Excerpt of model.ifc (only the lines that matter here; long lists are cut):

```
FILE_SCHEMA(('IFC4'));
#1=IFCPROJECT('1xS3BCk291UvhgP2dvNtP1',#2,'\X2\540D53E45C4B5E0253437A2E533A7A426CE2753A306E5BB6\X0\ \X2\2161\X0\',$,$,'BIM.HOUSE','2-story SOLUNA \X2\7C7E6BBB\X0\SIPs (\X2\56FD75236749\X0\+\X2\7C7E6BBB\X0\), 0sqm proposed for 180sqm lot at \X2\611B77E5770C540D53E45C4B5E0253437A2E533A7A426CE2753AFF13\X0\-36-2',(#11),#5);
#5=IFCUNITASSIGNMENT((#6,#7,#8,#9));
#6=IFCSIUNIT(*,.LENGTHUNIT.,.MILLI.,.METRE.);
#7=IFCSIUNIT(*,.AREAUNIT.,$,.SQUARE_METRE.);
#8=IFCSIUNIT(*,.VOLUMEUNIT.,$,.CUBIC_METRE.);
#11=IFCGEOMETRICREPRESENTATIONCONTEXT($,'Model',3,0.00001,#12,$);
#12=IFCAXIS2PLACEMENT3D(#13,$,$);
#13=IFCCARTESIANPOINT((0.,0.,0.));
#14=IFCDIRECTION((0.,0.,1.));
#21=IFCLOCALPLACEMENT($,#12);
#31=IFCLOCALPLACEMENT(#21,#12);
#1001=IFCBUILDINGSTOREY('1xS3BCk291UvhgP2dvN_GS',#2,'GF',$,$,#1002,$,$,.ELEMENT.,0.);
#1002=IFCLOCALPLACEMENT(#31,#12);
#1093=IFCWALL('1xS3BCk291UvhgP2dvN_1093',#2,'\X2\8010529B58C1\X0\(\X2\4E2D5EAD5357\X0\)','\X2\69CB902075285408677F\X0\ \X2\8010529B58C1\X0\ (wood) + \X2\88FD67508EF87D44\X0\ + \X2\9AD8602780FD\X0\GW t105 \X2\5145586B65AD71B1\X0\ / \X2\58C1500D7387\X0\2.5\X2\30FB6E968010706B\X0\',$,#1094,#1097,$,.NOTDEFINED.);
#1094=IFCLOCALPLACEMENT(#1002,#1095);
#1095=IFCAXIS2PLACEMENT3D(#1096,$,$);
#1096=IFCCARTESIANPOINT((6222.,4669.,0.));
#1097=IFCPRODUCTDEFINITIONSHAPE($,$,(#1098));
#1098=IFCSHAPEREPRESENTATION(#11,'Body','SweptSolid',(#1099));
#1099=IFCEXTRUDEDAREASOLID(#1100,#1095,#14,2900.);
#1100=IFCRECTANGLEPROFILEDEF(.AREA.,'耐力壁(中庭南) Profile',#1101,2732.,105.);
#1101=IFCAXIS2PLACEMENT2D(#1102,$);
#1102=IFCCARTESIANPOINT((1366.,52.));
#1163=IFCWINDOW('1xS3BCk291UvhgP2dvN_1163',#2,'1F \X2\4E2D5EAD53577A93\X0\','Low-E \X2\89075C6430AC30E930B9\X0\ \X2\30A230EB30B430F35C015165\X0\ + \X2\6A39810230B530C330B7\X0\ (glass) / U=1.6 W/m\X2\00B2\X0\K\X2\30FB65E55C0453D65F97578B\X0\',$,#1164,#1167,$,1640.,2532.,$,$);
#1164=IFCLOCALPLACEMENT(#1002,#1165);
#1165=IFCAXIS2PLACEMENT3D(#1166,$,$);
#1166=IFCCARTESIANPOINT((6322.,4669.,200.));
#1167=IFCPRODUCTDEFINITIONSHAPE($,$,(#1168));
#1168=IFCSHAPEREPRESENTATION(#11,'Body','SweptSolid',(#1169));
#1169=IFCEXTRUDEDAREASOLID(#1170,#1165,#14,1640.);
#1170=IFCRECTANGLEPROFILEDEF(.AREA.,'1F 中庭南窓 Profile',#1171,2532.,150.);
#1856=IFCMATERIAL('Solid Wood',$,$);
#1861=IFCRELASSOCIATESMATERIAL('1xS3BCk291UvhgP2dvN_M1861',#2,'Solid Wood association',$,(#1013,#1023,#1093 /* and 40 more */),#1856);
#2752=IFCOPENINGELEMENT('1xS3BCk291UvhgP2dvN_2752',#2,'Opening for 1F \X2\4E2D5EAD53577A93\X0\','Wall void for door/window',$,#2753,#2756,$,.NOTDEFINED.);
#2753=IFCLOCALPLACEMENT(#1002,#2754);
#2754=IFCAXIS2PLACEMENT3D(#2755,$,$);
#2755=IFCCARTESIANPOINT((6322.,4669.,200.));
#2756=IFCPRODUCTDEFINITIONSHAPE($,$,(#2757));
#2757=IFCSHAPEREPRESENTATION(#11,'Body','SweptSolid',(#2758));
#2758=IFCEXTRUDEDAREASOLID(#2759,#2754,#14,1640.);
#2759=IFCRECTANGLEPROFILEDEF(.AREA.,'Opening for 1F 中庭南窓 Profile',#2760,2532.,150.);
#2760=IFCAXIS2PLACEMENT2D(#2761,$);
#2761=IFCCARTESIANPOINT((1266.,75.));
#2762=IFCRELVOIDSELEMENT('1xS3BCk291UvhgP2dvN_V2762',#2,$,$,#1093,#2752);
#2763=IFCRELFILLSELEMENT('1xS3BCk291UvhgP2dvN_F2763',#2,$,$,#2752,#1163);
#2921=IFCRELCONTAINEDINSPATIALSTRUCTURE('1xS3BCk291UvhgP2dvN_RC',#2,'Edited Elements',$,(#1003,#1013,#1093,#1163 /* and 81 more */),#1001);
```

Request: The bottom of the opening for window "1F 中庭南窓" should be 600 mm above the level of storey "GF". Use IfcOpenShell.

```python
import numpy as np
import ifcopenshell
import ifcopenshell.api.geometry
import ifcopenshell.geom
import ifcopenshell.util.element
import ifcopenshell.util.placement
import ifcopenshell.util.shape
import ifcopenshell.util.unit

model = ifcopenshell.open("model.ifc")
unit_scale = ifcopenshell.util.unit.calculate_unit_scale(model)

window = model.by_id(1163)
opening = window.FillsVoids[0].RelatingOpeningElement
storey = ifcopenshell.util.element.get_container(window, ifc_class="IfcBuildingStorey")
level = ifcopenshell.util.placement.get_local_placement(storey.ObjectPlacement)[2, 3]

# The opening's origin need not be at the sill, so measure its lowest point.
shape = ifcopenshell.geom.create_shape(ifcopenshell.geom.settings(), opening)
bottom = ifcopenshell.util.shape.get_shape_bottom_elevation(shape, shape.geometry) / unit_scale
dz = level + 0.6 / unit_scale - bottom

shift = np.array([0.0, 0.0, dz])
# The window is not placed relative to its opening, so move both.
for product in (opening, window):
    matrix = ifcopenshell.util.placement.get_local_placement(product.ObjectPlacement)
    matrix[:3, 3] += shift
    ifcopenshell.api.geometry.edit_object_placement(model, product=product, matrix=matrix, is_si=False)

print(f"moved by {dz * unit_scale:+.3f} m")

model.write("model_edited.ifc")
```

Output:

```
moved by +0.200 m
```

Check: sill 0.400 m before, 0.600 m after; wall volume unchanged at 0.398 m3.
